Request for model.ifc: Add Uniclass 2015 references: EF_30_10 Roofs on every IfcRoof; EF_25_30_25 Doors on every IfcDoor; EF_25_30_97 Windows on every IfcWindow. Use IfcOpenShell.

First a look at what the model holds.

```python
import ifcopenshell

model = ifcopenshell.open("model.ifc")
print(model.schema)
print("classifications:", [c.Name for c in model.by_type("IfcClassification")])
for ifc_class in ("IfcDoor", "IfcRoof", "IfcStair", "IfcWall", "IfcWindow"):
    print(ifc_class, len(model.by_type(ifc_class)))
```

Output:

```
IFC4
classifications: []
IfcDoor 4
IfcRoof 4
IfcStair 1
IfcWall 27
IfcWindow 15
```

```python
import ifcopenshell
import ifcopenshell.api.classification

model = ifcopenshell.open("model.ifc")

system = ifcopenshell.api.classification.add_classification(model, classification="Uniclass 2015")

codes = {
    "IfcRoof": ("EF_30_10", "Roofs"),
    "IfcDoor": ("EF_25_30_25", "Doors"),
    "IfcWindow": ("EF_25_30_97", "Windows"),
}
for ifc_class, (code, name) in codes.items():
    products = model.by_type(ifc_class)
    ifcopenshell.api.classification.add_reference(
        model, products=products, classification=system, identification=code, name=name
    )
    print(code, len(products))

model.write("model-out.ifc")
```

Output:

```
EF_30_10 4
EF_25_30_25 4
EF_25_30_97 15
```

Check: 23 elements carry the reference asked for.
